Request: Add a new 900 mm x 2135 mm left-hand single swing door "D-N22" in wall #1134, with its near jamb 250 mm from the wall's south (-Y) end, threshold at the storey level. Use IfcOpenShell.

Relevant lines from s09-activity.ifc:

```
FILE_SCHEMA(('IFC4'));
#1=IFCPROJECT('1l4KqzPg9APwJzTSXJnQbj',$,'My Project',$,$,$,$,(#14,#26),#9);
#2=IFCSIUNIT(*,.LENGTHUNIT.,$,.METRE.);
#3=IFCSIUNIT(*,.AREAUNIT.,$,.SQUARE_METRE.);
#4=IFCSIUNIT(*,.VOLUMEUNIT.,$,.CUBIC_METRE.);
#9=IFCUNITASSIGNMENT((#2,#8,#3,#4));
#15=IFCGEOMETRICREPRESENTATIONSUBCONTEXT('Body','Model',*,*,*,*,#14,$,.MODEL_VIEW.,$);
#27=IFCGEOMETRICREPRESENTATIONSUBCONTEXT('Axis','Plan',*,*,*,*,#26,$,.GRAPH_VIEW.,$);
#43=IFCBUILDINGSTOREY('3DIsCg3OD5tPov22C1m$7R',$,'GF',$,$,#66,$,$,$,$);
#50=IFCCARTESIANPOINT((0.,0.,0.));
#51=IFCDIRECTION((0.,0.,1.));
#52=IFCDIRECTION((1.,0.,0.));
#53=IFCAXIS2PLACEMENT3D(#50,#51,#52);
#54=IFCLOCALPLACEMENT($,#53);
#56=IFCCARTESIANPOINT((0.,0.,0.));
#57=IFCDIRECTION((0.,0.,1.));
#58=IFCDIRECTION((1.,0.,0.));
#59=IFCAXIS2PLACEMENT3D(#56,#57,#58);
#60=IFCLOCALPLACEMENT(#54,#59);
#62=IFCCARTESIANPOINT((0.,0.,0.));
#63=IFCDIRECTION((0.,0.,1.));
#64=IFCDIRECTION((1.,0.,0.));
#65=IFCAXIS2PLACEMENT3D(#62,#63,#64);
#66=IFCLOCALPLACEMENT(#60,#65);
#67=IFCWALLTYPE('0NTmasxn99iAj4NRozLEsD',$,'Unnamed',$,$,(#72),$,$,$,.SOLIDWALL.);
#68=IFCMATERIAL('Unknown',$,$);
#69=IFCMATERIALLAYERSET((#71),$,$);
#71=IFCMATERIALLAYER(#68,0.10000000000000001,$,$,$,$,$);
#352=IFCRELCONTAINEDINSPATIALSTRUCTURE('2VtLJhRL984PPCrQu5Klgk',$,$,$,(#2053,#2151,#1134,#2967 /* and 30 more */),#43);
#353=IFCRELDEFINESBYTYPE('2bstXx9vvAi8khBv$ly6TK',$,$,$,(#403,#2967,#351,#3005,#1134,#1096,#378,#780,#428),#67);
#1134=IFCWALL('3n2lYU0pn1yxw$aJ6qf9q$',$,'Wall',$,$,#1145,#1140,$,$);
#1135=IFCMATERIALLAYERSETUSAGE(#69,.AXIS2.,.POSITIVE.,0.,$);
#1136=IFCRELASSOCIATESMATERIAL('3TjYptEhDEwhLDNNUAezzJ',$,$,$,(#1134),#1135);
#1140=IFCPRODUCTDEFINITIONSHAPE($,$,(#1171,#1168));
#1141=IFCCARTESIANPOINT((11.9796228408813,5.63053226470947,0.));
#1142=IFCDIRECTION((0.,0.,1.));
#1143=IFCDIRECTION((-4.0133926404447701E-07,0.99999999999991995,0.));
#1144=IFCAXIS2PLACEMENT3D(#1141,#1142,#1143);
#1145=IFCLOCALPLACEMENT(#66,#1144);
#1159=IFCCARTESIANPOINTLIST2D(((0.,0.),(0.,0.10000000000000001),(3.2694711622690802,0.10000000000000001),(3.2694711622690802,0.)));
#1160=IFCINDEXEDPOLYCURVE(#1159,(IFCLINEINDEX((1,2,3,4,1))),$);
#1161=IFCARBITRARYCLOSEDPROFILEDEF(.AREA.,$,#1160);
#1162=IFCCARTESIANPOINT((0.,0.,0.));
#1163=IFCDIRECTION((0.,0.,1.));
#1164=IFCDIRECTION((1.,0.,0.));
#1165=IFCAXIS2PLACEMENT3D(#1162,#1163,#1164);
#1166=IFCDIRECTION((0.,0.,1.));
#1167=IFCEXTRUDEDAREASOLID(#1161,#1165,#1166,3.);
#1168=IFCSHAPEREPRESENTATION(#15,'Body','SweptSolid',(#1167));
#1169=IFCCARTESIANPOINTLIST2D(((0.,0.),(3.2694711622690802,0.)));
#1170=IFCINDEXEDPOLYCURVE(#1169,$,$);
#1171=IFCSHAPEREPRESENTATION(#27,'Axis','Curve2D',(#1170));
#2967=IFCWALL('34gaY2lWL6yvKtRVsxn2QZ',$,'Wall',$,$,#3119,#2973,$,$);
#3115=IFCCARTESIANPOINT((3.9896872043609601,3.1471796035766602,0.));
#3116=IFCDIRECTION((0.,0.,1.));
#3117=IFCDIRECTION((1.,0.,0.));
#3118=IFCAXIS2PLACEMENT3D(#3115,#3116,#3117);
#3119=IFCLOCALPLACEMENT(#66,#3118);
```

```python
import numpy as np
import ifcopenshell
import ifcopenshell.api.feature
import ifcopenshell.api.geometry
import ifcopenshell.api.root
import ifcopenshell.api.spatial
import ifcopenshell.geom
import ifcopenshell.util.element
import ifcopenshell.util.placement
import ifcopenshell.util.representation
import ifcopenshell.util.shape
import ifcopenshell.util.unit

model = ifcopenshell.open("s09-activity.ifc")
unit_scale = ifcopenshell.util.unit.calculate_unit_scale(model)
settings = ifcopenshell.geom.settings()


def volume(element):
    """Net volume in cubic metres, openings subtracted."""
    shape = ifcopenshell.geom.create_shape(settings, element)
    return ifcopenshell.util.shape.get_volume(shape.geometry)


wall = model.by_guid("3n2lYU0pn1yxw$aJ6qf9q$")
storey = ifcopenshell.util.element.get_container(wall, ifc_class="IfcBuildingStorey")
context = ifcopenshell.util.representation.get_context(model, "Model", "Body", "MODEL_VIEW")
before = volume(wall)

width, height, from_end, sill = 0.9, 2.135, 0.25, 0.0  # metres

# The wall runs along its own X axis, and the end named is its -X end.
wall_shape = ifcopenshell.geom.create_shape(settings, wall)
x, y, z = ifcopenshell.util.shape.get_vertices(wall_shape.geometry).T
start = x.min() + from_end
face, thickness = float(y.min()), float(y.max() - y.min())
wall_matrix = ifcopenshell.util.placement.get_local_placement(wall.ObjectPlacement)
level = ifcopenshell.util.placement.get_local_placement(storey.ObjectPlacement)[2, 3]


def in_wall(x, y):
    """Placement at x, y metres in the wall's axes, at sill height."""
    matrix = wall_matrix.copy()
    matrix[:, 3] = wall_matrix @ np.array([x / unit_scale, y / unit_scale, 0.0, 1.0])
    matrix[2, 3] = level + sill / unit_scale
    return matrix


# Opening: a box that overshoots both wall faces by 50 mm.
opening = ifcopenshell.api.root.create_entity(model, ifc_class="IfcOpeningElement", predefined_type="OPENING")
box = ifcopenshell.api.geometry.add_wall_representation(
    model, context=context, length=width, height=height, thickness=thickness + 0.1
)
ifcopenshell.api.geometry.assign_representation(model, product=opening, representation=box)
ifcopenshell.api.geometry.edit_object_placement(model, product=opening, matrix=in_wall(start, face - 0.05), is_si=False)
ifcopenshell.api.feature.add_feature(model, feature=opening, element=wall)

door = ifcopenshell.api.root.create_entity(model, ifc_class="IfcDoor", name="D-N22", predefined_type="DOOR")
door.OverallWidth, door.OverallHeight = width / unit_scale, height / unit_scale
door.OperationType = "SINGLE_SWING_LEFT"
body = ifcopenshell.api.geometry.add_door_representation(
    model,
    context=context,
    overall_width=door.OverallWidth,
    overall_height=door.OverallHeight,
    operation_type="SINGLE_SWING_LEFT",
    lining_properties={"LiningDepth": thickness / unit_scale, "ThresholdDepth": thickness / unit_scale},
)
ifcopenshell.api.geometry.assign_representation(model, product=door, representation=body)
ifcopenshell.api.spatial.assign_container(model, products=[door], relating_structure=storey)
ifcopenshell.api.feature.add_filling(model, opening=opening, element=door)

# The lining spans the wall, so the door starts at the wall face.
ifcopenshell.api.geometry.edit_object_placement(model, product=door, matrix=in_wall(start, face), is_si=False)

after = volume(wall)

print(f"wall volume {before:.3f} -> {after:.3f} m3")

model.write("s09-activity-out.ifc")
```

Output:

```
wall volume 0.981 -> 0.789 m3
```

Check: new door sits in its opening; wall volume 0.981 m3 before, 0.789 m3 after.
